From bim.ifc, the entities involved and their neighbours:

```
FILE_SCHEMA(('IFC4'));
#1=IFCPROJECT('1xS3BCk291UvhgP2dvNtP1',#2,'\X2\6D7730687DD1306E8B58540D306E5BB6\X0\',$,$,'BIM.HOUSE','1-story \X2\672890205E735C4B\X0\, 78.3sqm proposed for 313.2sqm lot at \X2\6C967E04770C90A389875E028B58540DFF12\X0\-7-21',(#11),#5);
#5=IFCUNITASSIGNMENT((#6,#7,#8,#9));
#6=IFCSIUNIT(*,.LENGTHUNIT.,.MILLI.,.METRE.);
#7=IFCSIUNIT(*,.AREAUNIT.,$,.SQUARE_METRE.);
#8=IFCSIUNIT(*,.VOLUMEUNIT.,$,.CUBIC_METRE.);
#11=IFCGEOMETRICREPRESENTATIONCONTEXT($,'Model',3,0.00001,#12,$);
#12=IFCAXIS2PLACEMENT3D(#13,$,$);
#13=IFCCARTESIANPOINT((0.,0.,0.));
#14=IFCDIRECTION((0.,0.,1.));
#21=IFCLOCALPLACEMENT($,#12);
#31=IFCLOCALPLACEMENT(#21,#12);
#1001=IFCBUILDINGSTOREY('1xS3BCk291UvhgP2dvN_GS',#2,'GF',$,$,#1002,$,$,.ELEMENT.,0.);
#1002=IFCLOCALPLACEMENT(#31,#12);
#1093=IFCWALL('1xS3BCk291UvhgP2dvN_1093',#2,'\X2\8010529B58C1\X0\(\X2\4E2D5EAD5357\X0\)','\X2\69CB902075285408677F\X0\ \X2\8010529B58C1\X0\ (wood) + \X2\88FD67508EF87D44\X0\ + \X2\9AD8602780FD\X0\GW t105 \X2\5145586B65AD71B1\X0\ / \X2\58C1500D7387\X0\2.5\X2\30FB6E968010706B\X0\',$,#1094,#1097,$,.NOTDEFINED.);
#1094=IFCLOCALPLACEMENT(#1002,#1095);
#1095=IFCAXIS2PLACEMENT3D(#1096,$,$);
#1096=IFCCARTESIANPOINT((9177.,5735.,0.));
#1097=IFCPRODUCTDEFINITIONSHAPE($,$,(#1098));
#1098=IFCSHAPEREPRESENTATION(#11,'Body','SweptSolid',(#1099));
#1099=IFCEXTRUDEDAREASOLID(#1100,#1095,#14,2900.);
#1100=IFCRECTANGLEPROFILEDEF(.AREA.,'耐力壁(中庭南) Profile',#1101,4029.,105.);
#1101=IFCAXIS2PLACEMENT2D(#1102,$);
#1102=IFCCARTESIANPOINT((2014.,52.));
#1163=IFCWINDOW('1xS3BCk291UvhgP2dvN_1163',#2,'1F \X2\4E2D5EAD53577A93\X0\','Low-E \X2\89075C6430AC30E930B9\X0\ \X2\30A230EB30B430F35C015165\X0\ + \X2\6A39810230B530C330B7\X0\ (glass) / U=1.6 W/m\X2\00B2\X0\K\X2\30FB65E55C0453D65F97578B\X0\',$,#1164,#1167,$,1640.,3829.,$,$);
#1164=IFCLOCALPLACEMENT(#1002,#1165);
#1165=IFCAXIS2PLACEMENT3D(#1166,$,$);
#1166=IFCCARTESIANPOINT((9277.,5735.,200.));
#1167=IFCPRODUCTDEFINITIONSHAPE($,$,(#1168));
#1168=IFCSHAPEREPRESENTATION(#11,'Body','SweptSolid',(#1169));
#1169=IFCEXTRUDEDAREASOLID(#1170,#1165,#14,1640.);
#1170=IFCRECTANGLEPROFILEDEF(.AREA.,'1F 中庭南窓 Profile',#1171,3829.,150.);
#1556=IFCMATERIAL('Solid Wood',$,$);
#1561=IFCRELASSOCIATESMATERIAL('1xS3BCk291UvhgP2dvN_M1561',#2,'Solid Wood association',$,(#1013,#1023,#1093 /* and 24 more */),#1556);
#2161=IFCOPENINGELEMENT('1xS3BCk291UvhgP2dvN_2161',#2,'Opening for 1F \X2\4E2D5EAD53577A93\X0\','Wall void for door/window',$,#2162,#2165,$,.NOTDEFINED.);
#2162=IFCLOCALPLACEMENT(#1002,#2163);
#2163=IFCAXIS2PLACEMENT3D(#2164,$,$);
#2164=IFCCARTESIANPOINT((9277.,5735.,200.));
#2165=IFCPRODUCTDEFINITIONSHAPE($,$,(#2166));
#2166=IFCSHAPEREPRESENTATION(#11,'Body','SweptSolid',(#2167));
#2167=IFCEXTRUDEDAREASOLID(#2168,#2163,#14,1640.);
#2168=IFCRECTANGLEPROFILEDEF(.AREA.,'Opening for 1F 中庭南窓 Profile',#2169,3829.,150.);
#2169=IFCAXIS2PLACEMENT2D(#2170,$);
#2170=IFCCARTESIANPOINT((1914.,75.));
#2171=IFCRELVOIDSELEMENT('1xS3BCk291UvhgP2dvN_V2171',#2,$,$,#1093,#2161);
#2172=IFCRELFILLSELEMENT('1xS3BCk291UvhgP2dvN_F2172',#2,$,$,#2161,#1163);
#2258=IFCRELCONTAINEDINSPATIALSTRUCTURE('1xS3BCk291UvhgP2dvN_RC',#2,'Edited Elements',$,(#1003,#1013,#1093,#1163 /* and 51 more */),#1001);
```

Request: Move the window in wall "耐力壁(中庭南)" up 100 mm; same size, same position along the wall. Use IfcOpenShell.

```python
import numpy as np
import ifcopenshell
import ifcopenshell.api.geometry
import ifcopenshell.util.placement
import ifcopenshell.util.unit

model = ifcopenshell.open("bim.ifc")
unit_scale = ifcopenshell.util.unit.calculate_unit_scale(model)

window = model.by_guid("1xS3BCk291UvhgP2dvN_1163")
opening = window.FillsVoids[0].RelatingOpeningElement
dz = 0.1 / unit_scale

shift = np.array([0.0, 0.0, dz])
# The window is not placed relative to its opening, so move both.
for product in (opening, window):
    matrix = ifcopenshell.util.placement.get_local_placement(product.ObjectPlacement)
    matrix[:3, 3] += shift
    ifcopenshell.api.geometry.edit_object_placement(model, product=product, matrix=matrix, is_si=False)

print(f"moved by {dz * unit_scale:+.3f} m")

model.write("bim-out.ifc")
```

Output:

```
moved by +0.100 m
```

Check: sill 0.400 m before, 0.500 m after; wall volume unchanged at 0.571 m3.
